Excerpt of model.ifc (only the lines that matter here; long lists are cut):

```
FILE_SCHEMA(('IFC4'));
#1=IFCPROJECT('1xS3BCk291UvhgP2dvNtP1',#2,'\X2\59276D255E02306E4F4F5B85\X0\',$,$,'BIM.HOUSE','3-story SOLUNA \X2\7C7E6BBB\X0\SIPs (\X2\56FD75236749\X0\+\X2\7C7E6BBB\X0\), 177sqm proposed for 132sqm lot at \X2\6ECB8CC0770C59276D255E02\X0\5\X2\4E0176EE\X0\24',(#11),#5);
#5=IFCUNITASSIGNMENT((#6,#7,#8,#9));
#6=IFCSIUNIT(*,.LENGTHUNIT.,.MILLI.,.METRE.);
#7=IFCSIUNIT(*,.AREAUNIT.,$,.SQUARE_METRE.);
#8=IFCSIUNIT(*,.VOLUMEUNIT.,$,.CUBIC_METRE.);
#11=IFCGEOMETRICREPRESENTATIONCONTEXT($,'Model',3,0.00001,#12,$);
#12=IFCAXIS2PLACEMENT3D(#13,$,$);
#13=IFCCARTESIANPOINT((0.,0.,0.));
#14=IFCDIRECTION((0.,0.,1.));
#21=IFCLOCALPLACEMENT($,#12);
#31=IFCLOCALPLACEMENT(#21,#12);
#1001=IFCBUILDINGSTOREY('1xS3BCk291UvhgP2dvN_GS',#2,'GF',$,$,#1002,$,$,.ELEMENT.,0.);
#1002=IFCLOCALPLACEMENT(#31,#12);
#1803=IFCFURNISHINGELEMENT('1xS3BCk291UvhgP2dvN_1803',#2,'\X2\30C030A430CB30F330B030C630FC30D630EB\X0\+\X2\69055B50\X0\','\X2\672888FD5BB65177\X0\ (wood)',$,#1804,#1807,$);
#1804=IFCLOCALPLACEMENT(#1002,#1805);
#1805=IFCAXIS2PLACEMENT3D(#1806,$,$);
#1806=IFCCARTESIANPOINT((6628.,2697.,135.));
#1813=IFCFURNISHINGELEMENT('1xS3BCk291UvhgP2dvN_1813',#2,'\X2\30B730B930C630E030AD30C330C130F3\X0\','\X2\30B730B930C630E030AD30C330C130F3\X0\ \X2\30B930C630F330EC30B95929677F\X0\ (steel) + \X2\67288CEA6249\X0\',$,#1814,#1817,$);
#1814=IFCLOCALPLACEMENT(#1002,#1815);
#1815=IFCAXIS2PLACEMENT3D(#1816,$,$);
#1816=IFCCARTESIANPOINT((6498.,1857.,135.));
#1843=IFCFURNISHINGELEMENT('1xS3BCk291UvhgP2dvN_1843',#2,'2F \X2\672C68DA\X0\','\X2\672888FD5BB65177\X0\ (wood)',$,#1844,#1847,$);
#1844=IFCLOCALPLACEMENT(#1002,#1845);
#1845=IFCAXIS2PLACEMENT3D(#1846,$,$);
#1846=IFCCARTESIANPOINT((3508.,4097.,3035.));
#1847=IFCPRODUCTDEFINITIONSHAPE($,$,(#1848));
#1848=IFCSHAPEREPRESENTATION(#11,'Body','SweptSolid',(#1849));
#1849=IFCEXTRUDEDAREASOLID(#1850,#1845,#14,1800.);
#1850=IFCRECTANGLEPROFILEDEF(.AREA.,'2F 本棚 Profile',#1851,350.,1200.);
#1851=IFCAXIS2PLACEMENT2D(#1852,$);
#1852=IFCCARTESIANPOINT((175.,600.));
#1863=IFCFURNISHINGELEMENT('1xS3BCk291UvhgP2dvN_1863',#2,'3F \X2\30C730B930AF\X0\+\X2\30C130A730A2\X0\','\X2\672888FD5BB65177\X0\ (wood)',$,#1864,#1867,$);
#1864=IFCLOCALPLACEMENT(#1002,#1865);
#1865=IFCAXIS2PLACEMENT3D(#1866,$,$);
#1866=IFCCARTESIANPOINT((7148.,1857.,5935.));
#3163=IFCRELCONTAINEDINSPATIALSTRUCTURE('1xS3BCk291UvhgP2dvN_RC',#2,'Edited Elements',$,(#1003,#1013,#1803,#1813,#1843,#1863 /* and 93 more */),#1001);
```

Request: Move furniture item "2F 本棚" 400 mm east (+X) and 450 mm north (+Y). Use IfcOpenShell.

```python
import ifcopenshell
import ifcopenshell.api.geometry
import ifcopenshell.util.placement
import ifcopenshell.util.unit

model = ifcopenshell.open("model.ifc")
unit_scale = ifcopenshell.util.unit.calculate_unit_scale(model)

item = model.by_guid("1xS3BCk291UvhgP2dvN_1843")
matrix = ifcopenshell.util.placement.get_local_placement(item.ObjectPlacement)
matrix[0, 3] += 0.4 / unit_scale
matrix[1, 3] += 0.45 / unit_scale
ifcopenshell.api.geometry.edit_object_placement(model, product=item, matrix=matrix, is_si=False)

print(ifcopenshell.util.placement.get_local_placement(item.ObjectPlacement).round(3) + 0.0)

model.write("model-out.ifc")
```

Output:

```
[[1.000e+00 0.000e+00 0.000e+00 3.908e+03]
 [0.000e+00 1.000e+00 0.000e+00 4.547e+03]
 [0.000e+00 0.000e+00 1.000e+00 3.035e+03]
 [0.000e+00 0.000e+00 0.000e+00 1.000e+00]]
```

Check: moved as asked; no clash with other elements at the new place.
